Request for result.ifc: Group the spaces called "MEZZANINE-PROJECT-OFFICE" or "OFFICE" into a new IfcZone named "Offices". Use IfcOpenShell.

First a look at what the model holds.

```python
import ifcopenshell

model = ifcopenshell.open("result.ifc")
print(model.schema)
seen = {}
for space in model.by_type("IfcSpace"):
    seen[space.Name] = seen.get(space.Name, 0) + 1
for name, count in sorted(seen.items(), key=str):
    print(count, "x", name)
print("zones:", [z.Name for z in model.by_type("IfcZone")][:20])
```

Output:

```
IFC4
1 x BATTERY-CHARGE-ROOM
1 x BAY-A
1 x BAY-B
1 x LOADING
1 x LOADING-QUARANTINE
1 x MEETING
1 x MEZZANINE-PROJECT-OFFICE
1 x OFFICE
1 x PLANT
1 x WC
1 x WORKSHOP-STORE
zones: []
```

```python
import ifcopenshell
import ifcopenshell.api.group
import ifcopenshell.api.root

model = ifcopenshell.open("result.ifc")

names = {"MEZZANINE-PROJECT-OFFICE", "OFFICE"}
spaces = [s for s in model.by_type("IfcSpace") if s.Name in names]

zone = ifcopenshell.api.root.create_entity(model, ifc_class="IfcZone", name="Offices")
ifcopenshell.api.group.assign_group(model, products=spaces, group=zone)
print(len(spaces), "spaces in", zone.Name)

model.write("result_v2.ifc")
```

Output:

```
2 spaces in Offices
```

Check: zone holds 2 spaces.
